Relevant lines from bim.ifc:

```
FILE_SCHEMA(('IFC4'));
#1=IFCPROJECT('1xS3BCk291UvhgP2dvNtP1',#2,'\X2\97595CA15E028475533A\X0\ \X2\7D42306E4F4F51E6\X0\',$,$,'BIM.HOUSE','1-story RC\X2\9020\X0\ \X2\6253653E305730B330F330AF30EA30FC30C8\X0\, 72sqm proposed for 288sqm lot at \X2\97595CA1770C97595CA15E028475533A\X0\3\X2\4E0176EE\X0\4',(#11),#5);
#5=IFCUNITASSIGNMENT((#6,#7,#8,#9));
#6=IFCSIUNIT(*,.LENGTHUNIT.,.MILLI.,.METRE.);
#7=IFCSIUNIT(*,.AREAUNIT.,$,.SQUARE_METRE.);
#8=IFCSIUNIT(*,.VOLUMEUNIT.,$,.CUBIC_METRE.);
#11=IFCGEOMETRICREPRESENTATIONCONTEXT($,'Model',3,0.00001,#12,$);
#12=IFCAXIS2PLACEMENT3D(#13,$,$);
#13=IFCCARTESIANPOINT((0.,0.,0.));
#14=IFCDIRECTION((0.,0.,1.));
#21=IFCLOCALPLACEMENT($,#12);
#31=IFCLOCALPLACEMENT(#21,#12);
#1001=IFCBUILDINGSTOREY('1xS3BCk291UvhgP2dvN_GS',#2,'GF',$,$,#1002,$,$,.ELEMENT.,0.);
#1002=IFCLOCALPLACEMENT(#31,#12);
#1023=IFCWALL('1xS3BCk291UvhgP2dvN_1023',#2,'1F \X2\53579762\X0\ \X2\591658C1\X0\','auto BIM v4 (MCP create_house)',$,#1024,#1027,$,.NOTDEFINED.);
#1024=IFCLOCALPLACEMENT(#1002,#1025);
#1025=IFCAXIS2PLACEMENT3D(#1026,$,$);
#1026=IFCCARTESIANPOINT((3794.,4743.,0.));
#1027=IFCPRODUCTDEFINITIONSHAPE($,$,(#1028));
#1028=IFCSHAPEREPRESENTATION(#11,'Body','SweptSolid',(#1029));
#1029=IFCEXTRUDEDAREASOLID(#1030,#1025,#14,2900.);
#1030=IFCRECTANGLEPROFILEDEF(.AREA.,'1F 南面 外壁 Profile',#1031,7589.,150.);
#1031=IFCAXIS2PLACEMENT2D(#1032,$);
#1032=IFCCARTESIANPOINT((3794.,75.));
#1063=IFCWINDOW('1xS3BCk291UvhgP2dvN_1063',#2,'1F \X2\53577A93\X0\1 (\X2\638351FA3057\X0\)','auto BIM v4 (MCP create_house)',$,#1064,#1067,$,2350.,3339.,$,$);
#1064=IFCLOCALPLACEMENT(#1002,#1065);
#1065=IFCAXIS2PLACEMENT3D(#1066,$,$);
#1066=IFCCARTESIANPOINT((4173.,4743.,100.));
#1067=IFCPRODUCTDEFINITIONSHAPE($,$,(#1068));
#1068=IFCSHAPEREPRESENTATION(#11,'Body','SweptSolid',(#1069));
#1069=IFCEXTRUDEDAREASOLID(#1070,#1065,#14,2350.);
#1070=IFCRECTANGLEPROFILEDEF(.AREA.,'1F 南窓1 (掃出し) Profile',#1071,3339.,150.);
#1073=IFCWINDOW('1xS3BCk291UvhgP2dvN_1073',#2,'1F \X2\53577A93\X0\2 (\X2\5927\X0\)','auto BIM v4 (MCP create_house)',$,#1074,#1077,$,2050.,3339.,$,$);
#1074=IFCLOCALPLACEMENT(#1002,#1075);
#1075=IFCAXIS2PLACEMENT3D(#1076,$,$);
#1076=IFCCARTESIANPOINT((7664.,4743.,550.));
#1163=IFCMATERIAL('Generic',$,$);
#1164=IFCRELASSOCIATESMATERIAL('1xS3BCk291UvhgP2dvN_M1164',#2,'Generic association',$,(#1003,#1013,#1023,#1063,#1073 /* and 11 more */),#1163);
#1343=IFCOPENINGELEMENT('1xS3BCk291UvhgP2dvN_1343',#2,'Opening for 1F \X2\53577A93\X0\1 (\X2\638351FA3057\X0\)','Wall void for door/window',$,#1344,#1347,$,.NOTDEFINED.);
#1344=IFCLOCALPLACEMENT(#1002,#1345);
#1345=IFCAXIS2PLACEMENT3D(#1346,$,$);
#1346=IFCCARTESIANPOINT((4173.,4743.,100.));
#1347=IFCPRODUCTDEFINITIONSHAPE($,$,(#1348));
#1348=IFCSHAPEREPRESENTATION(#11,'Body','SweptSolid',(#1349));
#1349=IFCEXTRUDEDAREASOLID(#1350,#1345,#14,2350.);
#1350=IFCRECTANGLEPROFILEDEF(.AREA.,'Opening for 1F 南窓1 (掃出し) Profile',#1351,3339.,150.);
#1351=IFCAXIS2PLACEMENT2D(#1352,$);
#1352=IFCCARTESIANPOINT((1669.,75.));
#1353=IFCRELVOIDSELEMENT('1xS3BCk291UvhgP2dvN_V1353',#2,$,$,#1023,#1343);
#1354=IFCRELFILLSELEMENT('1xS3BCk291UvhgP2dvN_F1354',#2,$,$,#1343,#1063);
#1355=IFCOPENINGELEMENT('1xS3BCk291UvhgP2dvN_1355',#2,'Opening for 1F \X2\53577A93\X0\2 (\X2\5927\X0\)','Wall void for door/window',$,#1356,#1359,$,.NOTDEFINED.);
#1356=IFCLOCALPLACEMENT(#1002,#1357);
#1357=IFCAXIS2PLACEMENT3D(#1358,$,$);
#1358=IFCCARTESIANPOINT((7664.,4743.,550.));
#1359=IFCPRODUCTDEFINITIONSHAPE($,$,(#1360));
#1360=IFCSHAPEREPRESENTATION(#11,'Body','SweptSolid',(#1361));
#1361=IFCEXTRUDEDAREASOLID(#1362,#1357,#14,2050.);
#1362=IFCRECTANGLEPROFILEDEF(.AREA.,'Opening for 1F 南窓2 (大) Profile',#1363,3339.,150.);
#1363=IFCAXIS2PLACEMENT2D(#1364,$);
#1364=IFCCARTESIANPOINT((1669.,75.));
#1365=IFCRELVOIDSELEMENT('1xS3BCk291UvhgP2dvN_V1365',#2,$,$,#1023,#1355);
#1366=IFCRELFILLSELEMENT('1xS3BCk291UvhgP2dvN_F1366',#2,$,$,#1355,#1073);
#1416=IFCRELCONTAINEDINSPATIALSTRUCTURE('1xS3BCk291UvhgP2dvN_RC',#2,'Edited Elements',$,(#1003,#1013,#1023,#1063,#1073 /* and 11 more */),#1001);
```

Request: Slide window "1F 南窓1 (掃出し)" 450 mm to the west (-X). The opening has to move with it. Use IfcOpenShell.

```python
import ifcopenshell
import ifcopenshell.api.geometry
import ifcopenshell.util.placement
import ifcopenshell.util.unit

model = ifcopenshell.open("bim.ifc")
unit_scale = ifcopenshell.util.unit.calculate_unit_scale(model)

window = model.by_guid("1xS3BCk291UvhgP2dvN_1063")
opening = window.FillsVoids[0].RelatingOpeningElement
wall = opening.VoidsElements[0].RelatingBuildingElement

wall_matrix = ifcopenshell.util.placement.get_local_placement(wall.ObjectPlacement)
shift = wall_matrix[:3, 0] * -0.45 / unit_scale
before = ifcopenshell.util.placement.get_local_placement(window.ObjectPlacement)[:3, 3].copy()

# The window is not placed relative to its opening, so move both.
for product in (opening, window):
    matrix = ifcopenshell.util.placement.get_local_placement(product.ObjectPlacement)
    matrix[:3, 3] += shift
    ifcopenshell.api.geometry.edit_object_placement(model, product=product, matrix=matrix, is_si=False)

after = ifcopenshell.util.placement.get_local_placement(window.ObjectPlacement)[:3, 3]
print("window moved by", (after - before).round(3) + 0.0)

model.write("bim_updated.ifc")
```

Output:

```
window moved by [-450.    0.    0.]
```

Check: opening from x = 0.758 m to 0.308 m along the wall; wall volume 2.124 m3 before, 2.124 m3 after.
